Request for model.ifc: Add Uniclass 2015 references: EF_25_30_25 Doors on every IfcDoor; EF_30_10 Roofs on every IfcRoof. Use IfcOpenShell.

First a look at what the model holds.

```python
import ifcopenshell

model = ifcopenshell.open("model.ifc")
print(model.schema)
print("classifications:", [c.Name for c in model.by_type("IfcClassification")])
for ifc_class in ("IfcDoor", "IfcRoof", "IfcStair", "IfcWall", "IfcWindow"):
    print(ifc_class, len(model.by_type(ifc_class)))
```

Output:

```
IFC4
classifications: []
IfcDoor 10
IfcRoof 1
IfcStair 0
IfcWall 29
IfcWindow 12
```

```python
import ifcopenshell
import ifcopenshell.api.classification

model = ifcopenshell.open("model.ifc")

system = ifcopenshell.api.classification.add_classification(model, classification="Uniclass 2015")

codes = {
    "IfcDoor": ("EF_25_30_25", "Doors"),
    "IfcRoof": ("EF_30_10", "Roofs"),
}
for ifc_class, (code, name) in codes.items():
    products = model.by_type(ifc_class)
    ifcopenshell.api.classification.add_reference(
        model, products=products, classification=system, identification=code, name=name
    )
    print(code, len(products))

model.write("model_rev.ifc")
```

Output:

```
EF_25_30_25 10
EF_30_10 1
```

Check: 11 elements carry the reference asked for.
